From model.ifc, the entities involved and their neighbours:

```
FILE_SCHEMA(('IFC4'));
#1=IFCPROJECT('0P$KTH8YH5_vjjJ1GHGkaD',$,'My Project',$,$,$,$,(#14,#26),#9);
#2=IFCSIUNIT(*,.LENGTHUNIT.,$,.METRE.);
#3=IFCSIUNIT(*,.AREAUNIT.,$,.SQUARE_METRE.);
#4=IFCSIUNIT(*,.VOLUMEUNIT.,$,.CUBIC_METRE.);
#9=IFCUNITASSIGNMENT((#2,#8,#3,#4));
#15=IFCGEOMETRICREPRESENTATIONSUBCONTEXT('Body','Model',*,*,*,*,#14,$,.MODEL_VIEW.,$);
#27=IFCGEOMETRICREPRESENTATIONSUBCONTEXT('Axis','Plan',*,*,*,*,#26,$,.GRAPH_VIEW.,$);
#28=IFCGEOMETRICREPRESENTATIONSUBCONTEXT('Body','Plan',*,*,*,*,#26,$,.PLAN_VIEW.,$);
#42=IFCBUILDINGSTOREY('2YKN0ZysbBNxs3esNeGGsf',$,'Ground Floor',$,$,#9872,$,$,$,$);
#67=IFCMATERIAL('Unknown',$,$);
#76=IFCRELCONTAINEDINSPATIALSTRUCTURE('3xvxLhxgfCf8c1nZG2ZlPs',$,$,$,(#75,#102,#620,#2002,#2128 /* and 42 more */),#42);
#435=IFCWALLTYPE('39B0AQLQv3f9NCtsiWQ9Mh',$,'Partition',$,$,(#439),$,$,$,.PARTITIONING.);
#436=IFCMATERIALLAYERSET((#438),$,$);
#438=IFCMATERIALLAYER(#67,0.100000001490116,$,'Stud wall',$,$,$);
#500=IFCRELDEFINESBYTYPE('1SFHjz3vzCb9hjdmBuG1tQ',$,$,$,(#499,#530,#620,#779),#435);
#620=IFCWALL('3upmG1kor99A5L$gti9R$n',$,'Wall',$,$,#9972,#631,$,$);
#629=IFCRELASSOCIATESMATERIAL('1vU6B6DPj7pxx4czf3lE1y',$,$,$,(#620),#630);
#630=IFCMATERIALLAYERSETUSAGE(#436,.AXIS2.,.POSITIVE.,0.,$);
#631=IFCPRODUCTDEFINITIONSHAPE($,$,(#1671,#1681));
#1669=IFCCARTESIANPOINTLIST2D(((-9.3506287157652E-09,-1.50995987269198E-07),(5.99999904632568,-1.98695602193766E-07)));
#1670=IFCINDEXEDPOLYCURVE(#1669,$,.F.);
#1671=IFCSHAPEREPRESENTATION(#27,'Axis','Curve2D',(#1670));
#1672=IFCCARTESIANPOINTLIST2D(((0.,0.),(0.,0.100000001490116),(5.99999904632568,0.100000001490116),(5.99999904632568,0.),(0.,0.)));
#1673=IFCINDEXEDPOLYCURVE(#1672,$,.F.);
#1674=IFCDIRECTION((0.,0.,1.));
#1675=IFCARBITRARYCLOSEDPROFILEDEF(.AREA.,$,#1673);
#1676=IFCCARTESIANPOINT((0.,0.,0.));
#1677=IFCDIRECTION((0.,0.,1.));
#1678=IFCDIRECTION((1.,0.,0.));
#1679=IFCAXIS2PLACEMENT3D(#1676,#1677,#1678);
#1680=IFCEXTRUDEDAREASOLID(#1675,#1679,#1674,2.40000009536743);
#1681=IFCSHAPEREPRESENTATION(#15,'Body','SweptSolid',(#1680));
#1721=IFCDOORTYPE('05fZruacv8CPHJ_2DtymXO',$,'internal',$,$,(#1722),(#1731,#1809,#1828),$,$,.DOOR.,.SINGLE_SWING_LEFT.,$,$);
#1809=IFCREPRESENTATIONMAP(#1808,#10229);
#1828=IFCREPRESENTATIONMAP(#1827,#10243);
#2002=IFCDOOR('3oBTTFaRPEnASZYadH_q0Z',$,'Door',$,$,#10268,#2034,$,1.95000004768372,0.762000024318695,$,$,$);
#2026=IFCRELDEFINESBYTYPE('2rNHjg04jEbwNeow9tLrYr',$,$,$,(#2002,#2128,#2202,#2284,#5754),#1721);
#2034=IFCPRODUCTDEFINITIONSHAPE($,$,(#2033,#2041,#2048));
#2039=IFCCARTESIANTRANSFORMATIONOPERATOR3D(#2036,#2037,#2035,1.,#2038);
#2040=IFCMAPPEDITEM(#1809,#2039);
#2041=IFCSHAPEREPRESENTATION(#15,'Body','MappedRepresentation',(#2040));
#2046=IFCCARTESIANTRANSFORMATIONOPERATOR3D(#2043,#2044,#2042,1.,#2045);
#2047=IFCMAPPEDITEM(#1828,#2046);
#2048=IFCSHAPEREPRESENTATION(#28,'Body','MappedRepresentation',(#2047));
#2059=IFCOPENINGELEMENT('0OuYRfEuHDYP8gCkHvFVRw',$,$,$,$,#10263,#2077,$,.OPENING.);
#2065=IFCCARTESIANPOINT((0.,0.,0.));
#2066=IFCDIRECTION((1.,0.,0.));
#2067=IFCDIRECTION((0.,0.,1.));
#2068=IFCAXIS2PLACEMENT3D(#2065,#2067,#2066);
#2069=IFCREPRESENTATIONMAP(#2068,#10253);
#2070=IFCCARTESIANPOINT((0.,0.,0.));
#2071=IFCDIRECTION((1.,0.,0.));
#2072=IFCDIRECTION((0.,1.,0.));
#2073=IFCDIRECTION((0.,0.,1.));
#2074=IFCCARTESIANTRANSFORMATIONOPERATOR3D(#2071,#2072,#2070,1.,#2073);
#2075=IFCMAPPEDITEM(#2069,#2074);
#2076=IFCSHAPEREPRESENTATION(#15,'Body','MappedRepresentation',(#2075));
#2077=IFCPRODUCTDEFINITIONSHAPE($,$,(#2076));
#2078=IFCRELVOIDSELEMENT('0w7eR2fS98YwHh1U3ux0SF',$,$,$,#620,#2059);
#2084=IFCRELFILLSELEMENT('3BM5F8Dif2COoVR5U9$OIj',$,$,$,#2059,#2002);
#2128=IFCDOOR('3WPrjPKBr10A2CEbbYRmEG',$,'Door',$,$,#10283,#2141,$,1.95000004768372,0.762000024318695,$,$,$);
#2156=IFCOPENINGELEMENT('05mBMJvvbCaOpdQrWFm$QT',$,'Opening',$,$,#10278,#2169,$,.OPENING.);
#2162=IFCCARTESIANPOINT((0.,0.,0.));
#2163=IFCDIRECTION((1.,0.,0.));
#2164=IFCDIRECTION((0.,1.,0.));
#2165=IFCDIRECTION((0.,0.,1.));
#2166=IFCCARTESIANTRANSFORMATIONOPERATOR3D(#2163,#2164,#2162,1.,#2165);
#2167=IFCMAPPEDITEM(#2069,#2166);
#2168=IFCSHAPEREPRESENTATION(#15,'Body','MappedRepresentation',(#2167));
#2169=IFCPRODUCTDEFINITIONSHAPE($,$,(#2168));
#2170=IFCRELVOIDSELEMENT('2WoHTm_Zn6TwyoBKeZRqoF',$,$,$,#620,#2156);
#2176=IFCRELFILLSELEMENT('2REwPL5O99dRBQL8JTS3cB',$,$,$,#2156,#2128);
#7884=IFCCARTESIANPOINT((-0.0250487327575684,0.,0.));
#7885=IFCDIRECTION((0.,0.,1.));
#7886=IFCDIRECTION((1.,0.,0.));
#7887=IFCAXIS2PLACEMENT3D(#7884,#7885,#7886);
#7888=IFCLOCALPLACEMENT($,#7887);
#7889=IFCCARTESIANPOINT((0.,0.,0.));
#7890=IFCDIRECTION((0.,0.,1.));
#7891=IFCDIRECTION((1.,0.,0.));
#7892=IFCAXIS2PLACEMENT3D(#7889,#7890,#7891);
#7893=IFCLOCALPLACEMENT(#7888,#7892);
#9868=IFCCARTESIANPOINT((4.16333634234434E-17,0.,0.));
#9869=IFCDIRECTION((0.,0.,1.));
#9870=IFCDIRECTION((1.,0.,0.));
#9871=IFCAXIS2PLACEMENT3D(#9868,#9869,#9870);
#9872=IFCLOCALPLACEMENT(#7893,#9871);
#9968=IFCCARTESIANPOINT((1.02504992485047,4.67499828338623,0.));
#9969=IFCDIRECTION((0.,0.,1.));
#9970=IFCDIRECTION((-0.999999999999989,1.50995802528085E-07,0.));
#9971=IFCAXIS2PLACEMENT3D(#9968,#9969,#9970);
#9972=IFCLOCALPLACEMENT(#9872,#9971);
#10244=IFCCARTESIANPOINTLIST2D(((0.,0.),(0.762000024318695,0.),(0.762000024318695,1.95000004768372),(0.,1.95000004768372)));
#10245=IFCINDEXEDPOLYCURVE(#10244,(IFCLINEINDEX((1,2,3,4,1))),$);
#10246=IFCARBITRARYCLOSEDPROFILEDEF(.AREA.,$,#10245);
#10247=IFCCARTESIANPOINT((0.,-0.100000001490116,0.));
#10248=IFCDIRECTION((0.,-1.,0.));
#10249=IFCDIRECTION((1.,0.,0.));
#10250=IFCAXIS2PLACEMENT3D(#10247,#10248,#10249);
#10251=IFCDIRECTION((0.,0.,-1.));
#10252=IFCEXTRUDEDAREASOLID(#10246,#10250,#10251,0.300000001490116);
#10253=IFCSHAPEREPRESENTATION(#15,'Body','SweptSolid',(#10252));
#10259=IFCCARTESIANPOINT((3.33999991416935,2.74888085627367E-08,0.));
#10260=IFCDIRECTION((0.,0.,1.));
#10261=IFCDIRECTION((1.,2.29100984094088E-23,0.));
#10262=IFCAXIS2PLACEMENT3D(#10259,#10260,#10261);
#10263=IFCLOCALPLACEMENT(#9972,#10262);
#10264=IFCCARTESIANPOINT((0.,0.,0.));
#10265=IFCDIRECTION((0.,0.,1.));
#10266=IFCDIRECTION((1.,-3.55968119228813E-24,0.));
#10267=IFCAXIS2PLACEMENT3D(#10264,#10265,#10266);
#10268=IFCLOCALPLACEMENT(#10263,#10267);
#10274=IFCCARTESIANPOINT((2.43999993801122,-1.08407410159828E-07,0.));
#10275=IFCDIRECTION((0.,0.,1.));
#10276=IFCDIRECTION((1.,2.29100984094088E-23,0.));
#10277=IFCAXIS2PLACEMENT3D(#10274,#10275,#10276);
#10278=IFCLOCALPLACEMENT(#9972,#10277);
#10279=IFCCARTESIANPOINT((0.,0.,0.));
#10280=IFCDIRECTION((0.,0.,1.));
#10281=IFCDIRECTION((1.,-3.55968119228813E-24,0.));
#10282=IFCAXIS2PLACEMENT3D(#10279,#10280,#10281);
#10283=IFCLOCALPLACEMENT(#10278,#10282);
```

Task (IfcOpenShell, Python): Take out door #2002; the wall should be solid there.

```python
import ifcopenshell
import ifcopenshell.api.feature
import ifcopenshell.api.root
import ifcopenshell.geom
import ifcopenshell.util.shape

model = ifcopenshell.open("model.ifc")
settings = ifcopenshell.geom.settings()


def volume(element):
    """Net volume in cubic metres, openings subtracted."""
    shape = ifcopenshell.geom.create_shape(settings, element)
    return ifcopenshell.util.shape.get_volume(shape.geometry)


door = model.by_guid("3oBTTFaRPEnASZYadH_q0Z")
opening = door.FillsVoids[0].RelatingOpeningElement
wall = opening.VoidsElements[0].RelatingBuildingElement
before = volume(wall)

ifcopenshell.api.root.remove_product(model, product=door)
ifcopenshell.api.feature.remove_feature(model, feature=opening)

after = volume(wall)

print(f"wall volume {before:.3f} -> {after:.3f} m3")

model.write("model-out.ifc")
```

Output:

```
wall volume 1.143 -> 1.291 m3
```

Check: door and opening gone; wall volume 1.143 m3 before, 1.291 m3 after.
